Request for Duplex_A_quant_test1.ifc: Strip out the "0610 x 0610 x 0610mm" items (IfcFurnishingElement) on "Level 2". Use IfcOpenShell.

First a look at what the model holds.

```python
import ifcopenshell
import ifcopenshell.util.element

model = ifcopenshell.open("Duplex_A_quant_test1.ifc")
print(model.schema)
storey = next(s for s in model.by_type("IfcBuildingStorey") if s.Name == "Level 2")
furniture = [e for e in ifcopenshell.util.element.get_decomposition(storey) if e.is_a("IfcFurnishingElement")]
seen = {}
for e in furniture:
    element_type = ifcopenshell.util.element.get_type(e)
    name = element_type.Name if element_type not in (None, e) else None
    seen[name] = seen.get(name, 0) + 1
for name, count in sorted(seen.items(), key=str):
    print(count, "x", name)
```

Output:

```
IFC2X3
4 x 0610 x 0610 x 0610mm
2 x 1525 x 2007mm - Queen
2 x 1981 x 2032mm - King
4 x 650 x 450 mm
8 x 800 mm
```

```python
import ifcopenshell
import ifcopenshell.api.root
import ifcopenshell.util.element

model = ifcopenshell.open("Duplex_A_quant_test1.ifc")

storey = next(s for s in model.by_type("IfcBuildingStorey") if s.Name == "Level 2")
furniture = [e for e in ifcopenshell.util.element.get_decomposition(storey) if e.is_a("IfcFurnishingElement")]
targets = [e for e in furniture if (t := ifcopenshell.util.element.get_type(e)) not in (None, e) and t.Name == "0610 x 0610 x 0610mm"]

for e in targets:
    ifcopenshell.api.root.remove_product(model, product=e)
print(len(targets), "removed")

model.write("Duplex_A_quant_test1_rev.ifc")
```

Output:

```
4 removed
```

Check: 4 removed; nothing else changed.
